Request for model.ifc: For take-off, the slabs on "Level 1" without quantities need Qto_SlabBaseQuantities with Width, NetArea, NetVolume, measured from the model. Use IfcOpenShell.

First a look at what the model holds.

```python
import ifcopenshell
import ifcopenshell.util.element
import ifcopenshell.util.unit

model = ifcopenshell.open("model.ifc")
print(model.schema)
for unit_type in ("LENGTHUNIT", "AREAUNIT", "VOLUMEUNIT"):
    print(unit_type, ifcopenshell.util.unit.calculate_unit_scale(model, unit_type))
storey = next(s for s in model.by_type("IfcBuildingStorey") if s.Name == "Level 1")
slabs = [e for e in ifcopenshell.util.element.get_decomposition(storey) if e.is_a("IfcSlab")]
for e in sorted(slabs, key=lambda e: e.id()):
    print(e.id(), e.is_a(), e.Name, list(ifcopenshell.util.element.get_psets(e, qtos_only=True)), sep=" | ")
```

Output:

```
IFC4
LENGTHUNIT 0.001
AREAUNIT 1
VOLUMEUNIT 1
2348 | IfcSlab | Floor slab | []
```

```python
import ifcopenshell
import ifcopenshell.api.pset
import ifcopenshell.geom
import ifcopenshell.util.element
import ifcopenshell.util.shape
import ifcopenshell.util.unit

model = ifcopenshell.open("model.ifc")
unit_scale = ifcopenshell.util.unit.calculate_unit_scale(model)
area_scale = ifcopenshell.util.unit.calculate_unit_scale(model, "AREAUNIT")
volume_scale = ifcopenshell.util.unit.calculate_unit_scale(model, "VOLUMEUNIT")
settings = ifcopenshell.geom.settings()

storey = next(s for s in model.by_type("IfcBuildingStorey") if s.Name == "Level 1")
slabs = [e for e in ifcopenshell.util.element.get_decomposition(storey) if e.is_a("IfcSlab")]

for e in sorted(slabs, key=lambda e: e.id()):
    if ifcopenshell.util.element.get_psets(e, qtos_only=True, should_inherit=False):
        continue
    # Geometry comes back in metres, in the element's own axes.
    shape = ifcopenshell.geom.create_shape(settings, e)
    values = {
        "Width": ifcopenshell.util.shape.get_z(shape.geometry) / unit_scale,
        "NetArea": ifcopenshell.util.shape.get_footprint_area(shape.geometry) / area_scale,
        "NetVolume": ifcopenshell.util.shape.get_volume(shape.geometry) / volume_scale,
    }
    qto = ifcopenshell.api.pset.add_qto(model, product=e, name="Qto_SlabBaseQuantities")
    ifcopenshell.api.pset.edit_qto(model, qto=qto, properties=values)
    print(e.id(), {k: round(v, 3) for k, v in values.items()})

model.write("model_rev.ifc")
```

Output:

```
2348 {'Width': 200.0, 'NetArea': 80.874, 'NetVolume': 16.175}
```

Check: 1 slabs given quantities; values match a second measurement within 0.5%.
